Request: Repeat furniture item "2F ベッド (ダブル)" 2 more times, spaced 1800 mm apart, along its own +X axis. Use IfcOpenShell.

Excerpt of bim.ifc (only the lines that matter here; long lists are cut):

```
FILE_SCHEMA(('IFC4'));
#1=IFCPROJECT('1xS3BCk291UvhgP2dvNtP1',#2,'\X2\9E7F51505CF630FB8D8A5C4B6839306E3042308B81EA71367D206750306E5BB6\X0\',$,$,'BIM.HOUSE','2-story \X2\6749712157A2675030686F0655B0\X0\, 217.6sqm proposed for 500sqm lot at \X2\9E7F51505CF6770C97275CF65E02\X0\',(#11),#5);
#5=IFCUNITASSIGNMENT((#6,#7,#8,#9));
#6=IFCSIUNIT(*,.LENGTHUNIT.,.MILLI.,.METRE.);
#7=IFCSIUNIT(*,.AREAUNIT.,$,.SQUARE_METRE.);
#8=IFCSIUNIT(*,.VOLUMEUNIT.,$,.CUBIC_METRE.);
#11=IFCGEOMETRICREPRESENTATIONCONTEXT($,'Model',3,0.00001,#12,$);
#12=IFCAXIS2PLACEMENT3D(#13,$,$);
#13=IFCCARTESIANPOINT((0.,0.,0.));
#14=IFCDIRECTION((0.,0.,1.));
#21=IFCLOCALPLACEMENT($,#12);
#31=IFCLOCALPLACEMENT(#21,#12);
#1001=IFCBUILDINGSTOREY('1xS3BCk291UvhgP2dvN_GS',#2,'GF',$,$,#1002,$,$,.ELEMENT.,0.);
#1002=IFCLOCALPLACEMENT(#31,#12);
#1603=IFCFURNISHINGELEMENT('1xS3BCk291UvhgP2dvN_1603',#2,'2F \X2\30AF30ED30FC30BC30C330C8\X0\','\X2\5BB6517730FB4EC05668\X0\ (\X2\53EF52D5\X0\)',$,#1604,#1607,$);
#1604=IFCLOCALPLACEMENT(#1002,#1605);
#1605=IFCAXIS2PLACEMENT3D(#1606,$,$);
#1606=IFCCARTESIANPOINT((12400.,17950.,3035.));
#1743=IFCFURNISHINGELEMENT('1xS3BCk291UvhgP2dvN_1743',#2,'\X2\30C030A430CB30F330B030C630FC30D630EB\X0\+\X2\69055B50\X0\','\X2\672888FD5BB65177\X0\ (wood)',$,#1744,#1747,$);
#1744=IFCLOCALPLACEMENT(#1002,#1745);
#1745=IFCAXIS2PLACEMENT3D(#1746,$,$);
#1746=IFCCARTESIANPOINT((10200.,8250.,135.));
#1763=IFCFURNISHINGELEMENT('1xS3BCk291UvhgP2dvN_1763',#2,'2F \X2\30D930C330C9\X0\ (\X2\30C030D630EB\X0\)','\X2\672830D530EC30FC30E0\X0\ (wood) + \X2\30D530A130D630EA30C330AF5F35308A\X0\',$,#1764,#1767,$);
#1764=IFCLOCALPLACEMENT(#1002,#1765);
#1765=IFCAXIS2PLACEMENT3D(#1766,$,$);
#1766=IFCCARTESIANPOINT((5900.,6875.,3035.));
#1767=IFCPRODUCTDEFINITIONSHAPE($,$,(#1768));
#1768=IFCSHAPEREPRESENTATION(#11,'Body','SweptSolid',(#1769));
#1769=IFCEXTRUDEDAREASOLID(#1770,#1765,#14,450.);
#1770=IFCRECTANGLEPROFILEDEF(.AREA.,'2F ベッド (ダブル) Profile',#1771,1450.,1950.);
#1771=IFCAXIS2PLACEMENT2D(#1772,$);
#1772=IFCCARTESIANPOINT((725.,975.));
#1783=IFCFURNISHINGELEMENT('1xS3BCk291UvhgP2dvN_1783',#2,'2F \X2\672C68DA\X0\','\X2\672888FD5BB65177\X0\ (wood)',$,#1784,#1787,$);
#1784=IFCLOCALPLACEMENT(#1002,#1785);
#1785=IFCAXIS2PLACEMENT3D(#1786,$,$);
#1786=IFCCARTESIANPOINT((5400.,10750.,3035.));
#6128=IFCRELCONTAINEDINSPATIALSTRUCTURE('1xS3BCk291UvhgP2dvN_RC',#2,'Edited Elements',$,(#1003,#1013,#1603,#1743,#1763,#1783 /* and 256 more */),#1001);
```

```python
import ifcopenshell
import ifcopenshell.api.geometry
import ifcopenshell.api.root
import ifcopenshell.util.element
import ifcopenshell.util.placement
import ifcopenshell.util.unit

model = ifcopenshell.open("bim.ifc")
unit_scale = ifcopenshell.util.unit.calculate_unit_scale(model)


def reuse_history(source, copy):
    """copy_class also copies each property set's owner history, people and application; keep the originals."""
    for rel in copy.IsDefinedBy:
        if rel.is_a("IfcRelDefinesByProperties") and (history := rel.RelatingPropertyDefinition.OwnerHistory):
            rel.RelatingPropertyDefinition.OwnerHistory = source.OwnerHistory
            ifcopenshell.util.element.remove_deep2(model, history)


source = model.by_guid("1xS3BCk291UvhgP2dvN_1763")
base = ifcopenshell.util.placement.get_local_placement(source.ObjectPlacement)
step = base[:3, 0] * 1.8 / unit_scale

for i in range(1, 3):
    copy = ifcopenshell.api.root.copy_class(model, product=source)
    copy.Representation = ifcopenshell.util.element.copy_deep(
        model, source.Representation, exclude=["IfcGeometricRepresentationContext", "IfcRepresentationMap"]
    )
    reuse_history(source, copy)
    matrix = base.copy()
    matrix[:3, 3] += i * step
    print("added at", matrix[:3, 3].round(3) + 0.0)
    ifcopenshell.api.geometry.edit_object_placement(model, product=copy, matrix=matrix, is_si=False)

model.write("bim_edited.ifc")
```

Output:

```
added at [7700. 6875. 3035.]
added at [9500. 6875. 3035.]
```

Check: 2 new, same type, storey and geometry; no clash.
